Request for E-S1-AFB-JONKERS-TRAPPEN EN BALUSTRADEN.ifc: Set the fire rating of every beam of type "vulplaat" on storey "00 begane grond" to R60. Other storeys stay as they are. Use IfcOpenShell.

First a look at what the model holds.

```python
import ifcopenshell
import ifcopenshell.util.element

model = ifcopenshell.open("E-S1-AFB-JONKERS-TRAPPEN EN BALUSTRADEN.ifc")
print(model.schema)
storey = next(s for s in model.by_type("IfcBuildingStorey") if s.Name == "00 begane grond")
beams = [e for e in ifcopenshell.util.element.get_decomposition(storey) if e.is_a("IfcBeam")]
seen = {}
for e in beams:
    element_type = ifcopenshell.util.element.get_type(e)
    key = (element_type.Name if element_type != e and element_type else None, ifcopenshell.util.element.get_pset(e, "Pset_BeamCommon", "FireRating"))
    seen[key] = seen.get(key, 0) + 1
for (name, value), count in sorted(seen.items(), key=str):
    print(count, "x", name, "|", value)
```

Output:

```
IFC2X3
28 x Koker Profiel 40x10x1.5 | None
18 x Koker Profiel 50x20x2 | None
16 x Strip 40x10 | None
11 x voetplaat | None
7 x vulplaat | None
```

```python
import ifcopenshell
import ifcopenshell.api.pset
import ifcopenshell.util.element

model = ifcopenshell.open("E-S1-AFB-JONKERS-TRAPPEN EN BALUSTRADEN.ifc")

storey = next(s for s in model.by_type("IfcBuildingStorey") if s.Name == "00 begane grond")
beams = [e for e in ifcopenshell.util.element.get_decomposition(storey) if e.is_a("IfcBeam")]

count = 0
for e in beams:
    element_type = ifcopenshell.util.element.get_type(e)
    if element_type in (None, e) or element_type.Name != "vulplaat":
        continue
    # add_pset returns the element's existing set when there is one.
    pset = ifcopenshell.api.pset.add_pset(model, product=e, name="Pset_BeamCommon")
    ifcopenshell.api.pset.edit_pset(model, pset=pset, properties={"FireRating": "R60"})
    count += 1

print(count, "beams updated")

model.write("E-S1-AFB-JONKERS-TRAPPEN EN BALUSTRADEN_rev.ifc")
```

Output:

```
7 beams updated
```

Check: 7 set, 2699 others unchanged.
